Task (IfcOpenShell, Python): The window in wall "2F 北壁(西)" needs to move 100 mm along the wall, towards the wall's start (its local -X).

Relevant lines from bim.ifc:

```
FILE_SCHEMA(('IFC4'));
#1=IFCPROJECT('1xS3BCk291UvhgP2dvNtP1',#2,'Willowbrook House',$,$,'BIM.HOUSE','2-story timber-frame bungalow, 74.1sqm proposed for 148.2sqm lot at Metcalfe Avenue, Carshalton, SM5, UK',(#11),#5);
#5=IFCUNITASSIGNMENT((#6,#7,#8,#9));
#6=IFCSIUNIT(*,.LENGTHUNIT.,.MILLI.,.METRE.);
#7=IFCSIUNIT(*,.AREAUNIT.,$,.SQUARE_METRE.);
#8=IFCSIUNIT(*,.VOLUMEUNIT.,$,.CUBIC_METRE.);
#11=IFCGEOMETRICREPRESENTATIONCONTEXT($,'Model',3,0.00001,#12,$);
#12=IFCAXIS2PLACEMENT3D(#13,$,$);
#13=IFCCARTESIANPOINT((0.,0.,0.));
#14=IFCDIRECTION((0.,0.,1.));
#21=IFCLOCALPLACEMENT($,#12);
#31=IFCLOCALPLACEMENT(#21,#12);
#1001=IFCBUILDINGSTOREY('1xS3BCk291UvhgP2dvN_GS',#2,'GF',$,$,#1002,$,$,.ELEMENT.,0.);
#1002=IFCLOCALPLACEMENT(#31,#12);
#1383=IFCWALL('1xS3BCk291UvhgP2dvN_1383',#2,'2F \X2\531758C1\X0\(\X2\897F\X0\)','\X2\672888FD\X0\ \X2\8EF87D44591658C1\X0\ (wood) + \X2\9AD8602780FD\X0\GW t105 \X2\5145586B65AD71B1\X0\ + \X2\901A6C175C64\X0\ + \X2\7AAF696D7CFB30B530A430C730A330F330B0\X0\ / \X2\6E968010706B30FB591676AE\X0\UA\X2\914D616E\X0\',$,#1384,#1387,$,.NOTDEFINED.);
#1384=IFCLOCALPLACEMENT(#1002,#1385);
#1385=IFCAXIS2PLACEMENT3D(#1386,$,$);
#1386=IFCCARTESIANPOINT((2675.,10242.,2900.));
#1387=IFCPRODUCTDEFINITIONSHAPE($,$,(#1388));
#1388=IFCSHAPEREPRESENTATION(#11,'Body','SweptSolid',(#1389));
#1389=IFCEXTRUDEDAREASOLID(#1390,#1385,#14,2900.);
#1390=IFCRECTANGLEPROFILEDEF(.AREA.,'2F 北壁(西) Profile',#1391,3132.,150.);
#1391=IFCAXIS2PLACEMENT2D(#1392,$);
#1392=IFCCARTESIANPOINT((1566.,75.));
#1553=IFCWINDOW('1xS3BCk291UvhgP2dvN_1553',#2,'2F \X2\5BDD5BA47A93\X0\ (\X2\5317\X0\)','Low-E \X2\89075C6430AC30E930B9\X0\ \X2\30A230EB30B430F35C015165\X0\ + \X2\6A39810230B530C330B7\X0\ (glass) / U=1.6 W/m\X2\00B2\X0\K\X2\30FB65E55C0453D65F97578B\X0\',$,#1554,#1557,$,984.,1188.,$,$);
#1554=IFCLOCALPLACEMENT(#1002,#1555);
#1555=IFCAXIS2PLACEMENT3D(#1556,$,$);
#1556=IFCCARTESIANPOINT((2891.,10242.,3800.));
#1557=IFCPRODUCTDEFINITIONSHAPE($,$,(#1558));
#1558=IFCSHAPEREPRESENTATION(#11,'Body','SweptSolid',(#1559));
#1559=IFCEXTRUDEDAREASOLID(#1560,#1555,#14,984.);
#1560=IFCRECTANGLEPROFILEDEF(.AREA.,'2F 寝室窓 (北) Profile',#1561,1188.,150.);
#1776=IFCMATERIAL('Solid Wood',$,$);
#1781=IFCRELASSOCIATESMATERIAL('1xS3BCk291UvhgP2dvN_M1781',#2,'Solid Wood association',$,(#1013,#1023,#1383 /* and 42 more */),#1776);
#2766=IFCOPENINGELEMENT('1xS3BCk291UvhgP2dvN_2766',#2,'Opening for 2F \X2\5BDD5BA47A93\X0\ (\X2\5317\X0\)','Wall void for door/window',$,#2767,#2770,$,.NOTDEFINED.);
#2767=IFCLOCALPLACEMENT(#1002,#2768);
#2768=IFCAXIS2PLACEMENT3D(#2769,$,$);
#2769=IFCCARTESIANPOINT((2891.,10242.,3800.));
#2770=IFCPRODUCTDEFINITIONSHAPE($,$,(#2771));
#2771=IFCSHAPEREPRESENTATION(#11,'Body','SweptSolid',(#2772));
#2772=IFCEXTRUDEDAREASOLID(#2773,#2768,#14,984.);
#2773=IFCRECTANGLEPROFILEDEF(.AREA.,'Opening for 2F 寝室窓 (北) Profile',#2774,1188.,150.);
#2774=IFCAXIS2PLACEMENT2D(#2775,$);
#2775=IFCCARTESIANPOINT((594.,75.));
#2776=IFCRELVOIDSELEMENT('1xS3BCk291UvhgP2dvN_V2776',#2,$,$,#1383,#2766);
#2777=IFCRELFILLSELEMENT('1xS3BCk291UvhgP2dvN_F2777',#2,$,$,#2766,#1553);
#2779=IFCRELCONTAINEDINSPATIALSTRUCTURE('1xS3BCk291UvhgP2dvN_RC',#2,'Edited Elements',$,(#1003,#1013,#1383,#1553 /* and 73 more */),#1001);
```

```python
import ifcopenshell
import ifcopenshell.api.geometry
import ifcopenshell.util.placement
import ifcopenshell.util.unit

model = ifcopenshell.open("bim.ifc")
unit_scale = ifcopenshell.util.unit.calculate_unit_scale(model)

window = model.by_guid("1xS3BCk291UvhgP2dvN_1553")
opening = window.FillsVoids[0].RelatingOpeningElement
wall = opening.VoidsElements[0].RelatingBuildingElement

wall_matrix = ifcopenshell.util.placement.get_local_placement(wall.ObjectPlacement)
shift = wall_matrix[:3, 0] * -0.1 / unit_scale
before = ifcopenshell.util.placement.get_local_placement(window.ObjectPlacement)[:3, 3].copy()

# The window is not placed relative to its opening, so move both.
for product in (opening, window):
    matrix = ifcopenshell.util.placement.get_local_placement(product.ObjectPlacement)
    matrix[:3, 3] += shift
    ifcopenshell.api.geometry.edit_object_placement(model, product=product, matrix=matrix, is_si=False)

after = ifcopenshell.util.placement.get_local_placement(window.ObjectPlacement)[:3, 3]
print("window moved by", (after - before).round(3) + 0.0)

model.write("bim-out.ifc")
```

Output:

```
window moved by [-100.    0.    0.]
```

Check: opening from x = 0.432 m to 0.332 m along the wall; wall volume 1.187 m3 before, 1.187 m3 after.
